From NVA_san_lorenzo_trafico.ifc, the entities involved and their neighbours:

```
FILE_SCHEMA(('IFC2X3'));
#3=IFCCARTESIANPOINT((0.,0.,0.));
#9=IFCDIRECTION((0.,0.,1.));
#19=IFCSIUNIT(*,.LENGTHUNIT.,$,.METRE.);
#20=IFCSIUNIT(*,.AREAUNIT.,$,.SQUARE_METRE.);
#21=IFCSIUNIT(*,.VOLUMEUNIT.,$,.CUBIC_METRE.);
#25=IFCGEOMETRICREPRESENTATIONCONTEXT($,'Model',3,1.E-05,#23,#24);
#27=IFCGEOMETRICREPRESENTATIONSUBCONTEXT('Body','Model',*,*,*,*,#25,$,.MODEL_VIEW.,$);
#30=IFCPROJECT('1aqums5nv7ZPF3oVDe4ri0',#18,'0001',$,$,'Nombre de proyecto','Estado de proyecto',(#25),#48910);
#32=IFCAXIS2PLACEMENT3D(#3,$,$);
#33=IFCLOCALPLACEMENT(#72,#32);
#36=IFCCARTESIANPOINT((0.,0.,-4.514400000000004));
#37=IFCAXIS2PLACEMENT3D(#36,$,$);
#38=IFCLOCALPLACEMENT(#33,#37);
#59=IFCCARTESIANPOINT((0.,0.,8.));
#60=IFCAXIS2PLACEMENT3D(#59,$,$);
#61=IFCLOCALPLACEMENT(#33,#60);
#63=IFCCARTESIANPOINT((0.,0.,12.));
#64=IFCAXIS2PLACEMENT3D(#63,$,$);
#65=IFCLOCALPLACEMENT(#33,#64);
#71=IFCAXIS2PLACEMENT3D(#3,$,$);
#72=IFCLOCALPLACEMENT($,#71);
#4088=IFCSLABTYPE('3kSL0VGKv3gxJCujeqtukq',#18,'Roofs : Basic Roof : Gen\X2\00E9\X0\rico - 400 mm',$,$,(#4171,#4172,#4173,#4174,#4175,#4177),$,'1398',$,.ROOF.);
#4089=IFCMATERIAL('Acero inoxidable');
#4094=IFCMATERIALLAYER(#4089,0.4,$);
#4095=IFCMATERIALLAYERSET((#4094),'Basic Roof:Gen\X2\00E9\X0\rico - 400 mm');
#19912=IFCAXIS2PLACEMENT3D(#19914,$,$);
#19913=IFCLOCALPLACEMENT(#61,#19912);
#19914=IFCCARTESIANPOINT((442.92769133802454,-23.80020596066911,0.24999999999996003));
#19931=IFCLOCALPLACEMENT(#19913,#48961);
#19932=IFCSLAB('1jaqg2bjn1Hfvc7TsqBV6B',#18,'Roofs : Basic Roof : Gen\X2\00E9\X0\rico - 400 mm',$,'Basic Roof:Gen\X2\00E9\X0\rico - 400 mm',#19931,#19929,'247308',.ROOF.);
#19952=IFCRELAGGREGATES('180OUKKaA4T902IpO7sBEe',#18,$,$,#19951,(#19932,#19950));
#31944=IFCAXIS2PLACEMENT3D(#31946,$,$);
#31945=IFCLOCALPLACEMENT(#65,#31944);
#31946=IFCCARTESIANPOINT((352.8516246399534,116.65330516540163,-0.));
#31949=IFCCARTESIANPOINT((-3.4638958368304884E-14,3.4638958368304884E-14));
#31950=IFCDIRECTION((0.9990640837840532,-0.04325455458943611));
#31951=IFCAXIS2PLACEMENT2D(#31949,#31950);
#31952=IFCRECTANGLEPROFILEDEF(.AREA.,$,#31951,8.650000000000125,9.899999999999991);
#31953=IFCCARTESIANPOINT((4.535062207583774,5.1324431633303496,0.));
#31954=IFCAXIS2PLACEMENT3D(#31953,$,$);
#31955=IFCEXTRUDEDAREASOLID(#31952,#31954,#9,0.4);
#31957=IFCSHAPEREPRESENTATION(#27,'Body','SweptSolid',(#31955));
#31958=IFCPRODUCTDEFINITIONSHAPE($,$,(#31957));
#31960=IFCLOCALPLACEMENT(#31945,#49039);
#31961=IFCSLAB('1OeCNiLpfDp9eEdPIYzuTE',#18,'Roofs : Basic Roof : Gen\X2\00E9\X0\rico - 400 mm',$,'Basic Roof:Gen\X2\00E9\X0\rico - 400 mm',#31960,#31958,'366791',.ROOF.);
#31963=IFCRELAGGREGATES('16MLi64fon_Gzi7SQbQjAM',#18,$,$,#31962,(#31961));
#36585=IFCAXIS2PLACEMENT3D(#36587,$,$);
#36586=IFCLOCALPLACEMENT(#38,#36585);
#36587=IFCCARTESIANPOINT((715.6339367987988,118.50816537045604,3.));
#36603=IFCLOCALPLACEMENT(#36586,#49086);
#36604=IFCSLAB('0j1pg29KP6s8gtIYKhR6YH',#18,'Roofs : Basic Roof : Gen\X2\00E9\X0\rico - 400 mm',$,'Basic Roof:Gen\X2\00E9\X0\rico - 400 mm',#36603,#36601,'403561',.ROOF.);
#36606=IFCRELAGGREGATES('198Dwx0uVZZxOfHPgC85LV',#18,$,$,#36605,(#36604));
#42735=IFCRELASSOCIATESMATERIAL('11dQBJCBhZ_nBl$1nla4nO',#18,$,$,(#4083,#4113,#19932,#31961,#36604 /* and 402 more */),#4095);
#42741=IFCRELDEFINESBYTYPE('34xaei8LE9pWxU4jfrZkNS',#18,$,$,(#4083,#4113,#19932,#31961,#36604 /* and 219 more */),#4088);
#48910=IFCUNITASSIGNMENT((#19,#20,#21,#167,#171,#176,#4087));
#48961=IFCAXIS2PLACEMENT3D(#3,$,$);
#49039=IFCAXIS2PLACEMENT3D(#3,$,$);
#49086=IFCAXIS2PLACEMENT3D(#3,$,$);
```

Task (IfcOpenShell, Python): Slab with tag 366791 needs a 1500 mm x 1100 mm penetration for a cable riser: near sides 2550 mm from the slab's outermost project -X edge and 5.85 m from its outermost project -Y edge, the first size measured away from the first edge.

```python
import numpy as np
import ifcopenshell
import ifcopenshell.api.feature
import ifcopenshell.api.geometry
import ifcopenshell.api.root
import ifcopenshell.geom
import ifcopenshell.util.placement
import ifcopenshell.util.representation
import ifcopenshell.util.shape
import ifcopenshell.util.unit

model = ifcopenshell.open("NVA_san_lorenzo_trafico.ifc")
unit_scale = ifcopenshell.util.unit.calculate_unit_scale(model)
settings = ifcopenshell.geom.settings()


def volume(element):
    """Net volume in cubic metres, openings subtracted."""
    shape = ifcopenshell.geom.create_shape(settings, element)
    return ifcopenshell.util.shape.get_volume(shape.geometry)


slab = model.by_guid("1OeCNiLpfDp9eEdPIYzuTE")
before = volume(slab)

# Extent in the slab's own axes, in metres. The edges named are its -X and -Y sides.
slab_shape = ifcopenshell.geom.create_shape(settings, slab)
vertices = ifcopenshell.util.shape.get_vertices(slab_shape.geometry)
x_min, y_min, bottom = vertices.min(axis=0)
top = vertices[:, 2].max()

opening = ifcopenshell.api.root.create_entity(model, ifc_class="IfcOpeningElement", name="Cable riser opening")
context = ifcopenshell.util.representation.get_context(model, "Model", "Body", "MODEL_VIEW")
width, depth = 1.5, 1.1
outline = [(0.0, 0.0), (width, 0.0), (width, depth), (0.0, depth), (0.0, 0.0)]
# Overshoot both faces by 50 mm so the cut is clean.
shape = ifcopenshell.api.geometry.add_slab_representation(
    model, context=context, depth=top - bottom + 0.1, polyline=outline
)
ifcopenshell.api.geometry.assign_representation(model, product=opening, representation=shape)

matrix = ifcopenshell.util.placement.get_local_placement(slab.ObjectPlacement)
matrix[:, 3] = matrix @ np.append(np.array([x_min + 2.55, y_min + 5.85, bottom - 0.05]) / unit_scale, 1.0)
ifcopenshell.api.geometry.edit_object_placement(model, product=opening, matrix=matrix, is_si=False)
ifcopenshell.api.feature.add_feature(model, feature=opening, element=slab)

after = volume(slab)

print(f"slab volume {before:.3f} -> {after:.3f} m3")

model.write("NVA_san_lorenzo_trafico_rev.ifc")
```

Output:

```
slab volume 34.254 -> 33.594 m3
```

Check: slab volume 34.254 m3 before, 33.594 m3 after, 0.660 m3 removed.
